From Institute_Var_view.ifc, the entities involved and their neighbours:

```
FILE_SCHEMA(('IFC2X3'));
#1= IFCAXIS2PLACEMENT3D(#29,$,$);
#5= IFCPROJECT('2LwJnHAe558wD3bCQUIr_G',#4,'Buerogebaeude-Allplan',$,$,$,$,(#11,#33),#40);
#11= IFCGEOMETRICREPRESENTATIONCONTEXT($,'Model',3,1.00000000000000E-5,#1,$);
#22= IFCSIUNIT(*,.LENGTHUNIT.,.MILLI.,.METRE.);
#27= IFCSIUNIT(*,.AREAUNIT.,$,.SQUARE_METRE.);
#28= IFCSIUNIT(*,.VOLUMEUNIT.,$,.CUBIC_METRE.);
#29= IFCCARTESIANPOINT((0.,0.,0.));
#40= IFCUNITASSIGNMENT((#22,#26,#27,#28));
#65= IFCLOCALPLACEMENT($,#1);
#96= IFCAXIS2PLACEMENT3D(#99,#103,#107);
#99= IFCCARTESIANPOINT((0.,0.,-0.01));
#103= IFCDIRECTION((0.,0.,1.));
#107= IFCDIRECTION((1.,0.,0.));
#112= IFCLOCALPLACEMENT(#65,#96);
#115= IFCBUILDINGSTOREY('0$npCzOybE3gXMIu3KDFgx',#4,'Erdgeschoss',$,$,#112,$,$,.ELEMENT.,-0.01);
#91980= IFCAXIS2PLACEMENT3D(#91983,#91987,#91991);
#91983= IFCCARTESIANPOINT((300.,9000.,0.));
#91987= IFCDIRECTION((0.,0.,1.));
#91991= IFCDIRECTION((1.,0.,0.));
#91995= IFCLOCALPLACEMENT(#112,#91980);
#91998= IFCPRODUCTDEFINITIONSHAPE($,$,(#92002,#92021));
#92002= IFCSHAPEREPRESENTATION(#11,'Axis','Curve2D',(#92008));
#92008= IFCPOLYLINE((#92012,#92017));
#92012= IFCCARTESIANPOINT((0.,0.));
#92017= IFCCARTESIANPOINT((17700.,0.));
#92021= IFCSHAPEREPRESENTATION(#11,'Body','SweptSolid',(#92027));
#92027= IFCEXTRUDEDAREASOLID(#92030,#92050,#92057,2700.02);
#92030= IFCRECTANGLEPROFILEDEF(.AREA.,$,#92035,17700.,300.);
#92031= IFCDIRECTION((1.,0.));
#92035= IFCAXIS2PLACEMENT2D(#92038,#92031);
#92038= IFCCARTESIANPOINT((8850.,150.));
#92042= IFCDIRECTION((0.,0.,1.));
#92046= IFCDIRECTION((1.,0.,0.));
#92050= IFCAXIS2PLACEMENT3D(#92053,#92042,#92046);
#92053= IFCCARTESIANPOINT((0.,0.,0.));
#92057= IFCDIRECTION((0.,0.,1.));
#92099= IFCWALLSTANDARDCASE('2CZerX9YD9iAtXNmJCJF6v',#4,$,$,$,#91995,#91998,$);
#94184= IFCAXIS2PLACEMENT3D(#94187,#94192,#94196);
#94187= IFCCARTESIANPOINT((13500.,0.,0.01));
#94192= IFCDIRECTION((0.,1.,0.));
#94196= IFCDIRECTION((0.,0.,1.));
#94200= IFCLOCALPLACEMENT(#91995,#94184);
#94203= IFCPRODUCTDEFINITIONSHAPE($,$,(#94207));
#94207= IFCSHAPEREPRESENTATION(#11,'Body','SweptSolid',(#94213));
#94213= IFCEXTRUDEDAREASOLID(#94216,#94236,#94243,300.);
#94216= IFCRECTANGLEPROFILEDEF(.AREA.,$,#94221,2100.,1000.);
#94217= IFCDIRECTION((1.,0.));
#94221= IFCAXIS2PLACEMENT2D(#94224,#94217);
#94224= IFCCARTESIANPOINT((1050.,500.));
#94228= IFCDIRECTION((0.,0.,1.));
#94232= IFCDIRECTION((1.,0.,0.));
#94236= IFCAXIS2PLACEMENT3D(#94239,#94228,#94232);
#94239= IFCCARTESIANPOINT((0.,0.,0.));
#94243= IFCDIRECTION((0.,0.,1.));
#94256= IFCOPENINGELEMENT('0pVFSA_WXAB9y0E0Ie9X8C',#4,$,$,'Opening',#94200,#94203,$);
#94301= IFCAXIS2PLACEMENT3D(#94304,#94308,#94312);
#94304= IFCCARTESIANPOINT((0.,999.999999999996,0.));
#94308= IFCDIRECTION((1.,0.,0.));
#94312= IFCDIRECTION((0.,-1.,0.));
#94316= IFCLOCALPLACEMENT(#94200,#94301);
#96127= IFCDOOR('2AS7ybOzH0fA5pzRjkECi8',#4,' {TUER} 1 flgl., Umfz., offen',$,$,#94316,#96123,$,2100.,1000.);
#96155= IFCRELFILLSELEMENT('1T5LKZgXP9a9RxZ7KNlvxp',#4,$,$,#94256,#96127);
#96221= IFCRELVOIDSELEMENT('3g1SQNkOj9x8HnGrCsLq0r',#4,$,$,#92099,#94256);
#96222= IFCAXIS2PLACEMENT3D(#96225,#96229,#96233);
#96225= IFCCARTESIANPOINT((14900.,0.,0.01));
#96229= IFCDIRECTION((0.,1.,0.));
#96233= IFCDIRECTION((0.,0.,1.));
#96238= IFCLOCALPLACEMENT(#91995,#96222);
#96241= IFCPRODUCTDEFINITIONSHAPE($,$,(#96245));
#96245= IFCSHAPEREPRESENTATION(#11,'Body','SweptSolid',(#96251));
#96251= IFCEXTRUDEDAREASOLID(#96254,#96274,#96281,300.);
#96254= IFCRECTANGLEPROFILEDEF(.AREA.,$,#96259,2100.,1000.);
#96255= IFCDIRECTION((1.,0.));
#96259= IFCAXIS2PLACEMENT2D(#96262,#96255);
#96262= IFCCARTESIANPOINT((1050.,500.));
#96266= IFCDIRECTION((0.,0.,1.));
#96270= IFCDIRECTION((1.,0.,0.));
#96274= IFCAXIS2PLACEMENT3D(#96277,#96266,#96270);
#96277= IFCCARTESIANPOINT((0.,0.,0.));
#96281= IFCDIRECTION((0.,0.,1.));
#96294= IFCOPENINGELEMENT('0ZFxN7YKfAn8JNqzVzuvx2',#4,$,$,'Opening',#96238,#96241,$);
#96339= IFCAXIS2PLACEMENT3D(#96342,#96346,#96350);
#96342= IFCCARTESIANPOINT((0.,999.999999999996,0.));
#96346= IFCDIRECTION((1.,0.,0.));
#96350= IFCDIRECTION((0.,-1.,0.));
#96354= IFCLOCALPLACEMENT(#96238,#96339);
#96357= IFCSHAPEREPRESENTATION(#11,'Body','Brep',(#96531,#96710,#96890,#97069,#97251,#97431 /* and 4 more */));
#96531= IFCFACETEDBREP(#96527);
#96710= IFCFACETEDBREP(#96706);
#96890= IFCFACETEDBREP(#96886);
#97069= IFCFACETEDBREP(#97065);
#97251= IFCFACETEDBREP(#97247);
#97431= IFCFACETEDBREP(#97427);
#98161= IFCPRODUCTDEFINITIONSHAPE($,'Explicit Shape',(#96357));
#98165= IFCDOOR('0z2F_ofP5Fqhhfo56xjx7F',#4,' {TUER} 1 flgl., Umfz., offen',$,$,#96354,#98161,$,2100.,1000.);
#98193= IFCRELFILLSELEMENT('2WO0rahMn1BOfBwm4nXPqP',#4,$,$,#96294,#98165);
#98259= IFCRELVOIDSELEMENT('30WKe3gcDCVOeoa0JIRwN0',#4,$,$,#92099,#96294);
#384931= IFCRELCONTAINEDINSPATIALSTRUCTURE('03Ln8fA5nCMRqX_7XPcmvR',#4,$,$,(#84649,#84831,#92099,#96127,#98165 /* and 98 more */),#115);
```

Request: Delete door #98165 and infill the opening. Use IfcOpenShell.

```python
import ifcopenshell
import ifcopenshell.api.feature
import ifcopenshell.api.root
import ifcopenshell.geom
import ifcopenshell.util.shape

model = ifcopenshell.open("Institute_Var_view.ifc")
settings = ifcopenshell.geom.settings()


def volume(element):
    """Net volume in cubic metres, openings subtracted."""
    shape = ifcopenshell.geom.create_shape(settings, element)
    return ifcopenshell.util.shape.get_volume(shape.geometry)


door = model.by_guid("0z2F_ofP5Fqhhfo56xjx7F")
opening = door.FillsVoids[0].RelatingOpeningElement
wall = opening.VoidsElements[0].RelatingBuildingElement
before = volume(wall)

ifcopenshell.api.root.remove_product(model, product=door)
ifcopenshell.api.feature.remove_feature(model, feature=opening)

after = volume(wall)

print(f"wall volume {before:.3f} -> {after:.3f} m3")

model.write("Institute_Var_view_rev.ifc")
```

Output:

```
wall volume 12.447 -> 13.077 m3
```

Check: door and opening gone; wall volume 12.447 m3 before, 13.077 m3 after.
